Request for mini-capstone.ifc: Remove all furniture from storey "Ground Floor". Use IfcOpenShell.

First a look at what the model holds.

```python
import ifcopenshell
import ifcopenshell.util.element

model = ifcopenshell.open("mini-capstone.ifc")
print(model.schema)
storey = next(s for s in model.by_type("IfcBuildingStorey") if s.Name == "Ground Floor")
furniture = [e for e in ifcopenshell.util.element.get_decomposition(storey) if e.is_a("IfcFurnishingElement")]
seen = {}
for e in furniture:
    element_type = ifcopenshell.util.element.get_type(e)
    name = element_type.Name if element_type not in (None, e) else None
    seen[name] = seen.get(name, 0) + 1
for name, count in sorted(seen.items(), key=str):
    print(count, "x", name)
```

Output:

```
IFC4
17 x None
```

```python
import ifcopenshell
import ifcopenshell.api.root
import ifcopenshell.util.element

model = ifcopenshell.open("mini-capstone.ifc")

storey = next(s for s in model.by_type("IfcBuildingStorey") if s.Name == "Ground Floor")
furniture = [e for e in ifcopenshell.util.element.get_decomposition(storey) if e.is_a("IfcFurnishingElement")]

for e in furniture:
    ifcopenshell.api.root.remove_product(model, product=e)
print(len(furniture), "removed")

model.write("mini-capstone_v2.ifc")
```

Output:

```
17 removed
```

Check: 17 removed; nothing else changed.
